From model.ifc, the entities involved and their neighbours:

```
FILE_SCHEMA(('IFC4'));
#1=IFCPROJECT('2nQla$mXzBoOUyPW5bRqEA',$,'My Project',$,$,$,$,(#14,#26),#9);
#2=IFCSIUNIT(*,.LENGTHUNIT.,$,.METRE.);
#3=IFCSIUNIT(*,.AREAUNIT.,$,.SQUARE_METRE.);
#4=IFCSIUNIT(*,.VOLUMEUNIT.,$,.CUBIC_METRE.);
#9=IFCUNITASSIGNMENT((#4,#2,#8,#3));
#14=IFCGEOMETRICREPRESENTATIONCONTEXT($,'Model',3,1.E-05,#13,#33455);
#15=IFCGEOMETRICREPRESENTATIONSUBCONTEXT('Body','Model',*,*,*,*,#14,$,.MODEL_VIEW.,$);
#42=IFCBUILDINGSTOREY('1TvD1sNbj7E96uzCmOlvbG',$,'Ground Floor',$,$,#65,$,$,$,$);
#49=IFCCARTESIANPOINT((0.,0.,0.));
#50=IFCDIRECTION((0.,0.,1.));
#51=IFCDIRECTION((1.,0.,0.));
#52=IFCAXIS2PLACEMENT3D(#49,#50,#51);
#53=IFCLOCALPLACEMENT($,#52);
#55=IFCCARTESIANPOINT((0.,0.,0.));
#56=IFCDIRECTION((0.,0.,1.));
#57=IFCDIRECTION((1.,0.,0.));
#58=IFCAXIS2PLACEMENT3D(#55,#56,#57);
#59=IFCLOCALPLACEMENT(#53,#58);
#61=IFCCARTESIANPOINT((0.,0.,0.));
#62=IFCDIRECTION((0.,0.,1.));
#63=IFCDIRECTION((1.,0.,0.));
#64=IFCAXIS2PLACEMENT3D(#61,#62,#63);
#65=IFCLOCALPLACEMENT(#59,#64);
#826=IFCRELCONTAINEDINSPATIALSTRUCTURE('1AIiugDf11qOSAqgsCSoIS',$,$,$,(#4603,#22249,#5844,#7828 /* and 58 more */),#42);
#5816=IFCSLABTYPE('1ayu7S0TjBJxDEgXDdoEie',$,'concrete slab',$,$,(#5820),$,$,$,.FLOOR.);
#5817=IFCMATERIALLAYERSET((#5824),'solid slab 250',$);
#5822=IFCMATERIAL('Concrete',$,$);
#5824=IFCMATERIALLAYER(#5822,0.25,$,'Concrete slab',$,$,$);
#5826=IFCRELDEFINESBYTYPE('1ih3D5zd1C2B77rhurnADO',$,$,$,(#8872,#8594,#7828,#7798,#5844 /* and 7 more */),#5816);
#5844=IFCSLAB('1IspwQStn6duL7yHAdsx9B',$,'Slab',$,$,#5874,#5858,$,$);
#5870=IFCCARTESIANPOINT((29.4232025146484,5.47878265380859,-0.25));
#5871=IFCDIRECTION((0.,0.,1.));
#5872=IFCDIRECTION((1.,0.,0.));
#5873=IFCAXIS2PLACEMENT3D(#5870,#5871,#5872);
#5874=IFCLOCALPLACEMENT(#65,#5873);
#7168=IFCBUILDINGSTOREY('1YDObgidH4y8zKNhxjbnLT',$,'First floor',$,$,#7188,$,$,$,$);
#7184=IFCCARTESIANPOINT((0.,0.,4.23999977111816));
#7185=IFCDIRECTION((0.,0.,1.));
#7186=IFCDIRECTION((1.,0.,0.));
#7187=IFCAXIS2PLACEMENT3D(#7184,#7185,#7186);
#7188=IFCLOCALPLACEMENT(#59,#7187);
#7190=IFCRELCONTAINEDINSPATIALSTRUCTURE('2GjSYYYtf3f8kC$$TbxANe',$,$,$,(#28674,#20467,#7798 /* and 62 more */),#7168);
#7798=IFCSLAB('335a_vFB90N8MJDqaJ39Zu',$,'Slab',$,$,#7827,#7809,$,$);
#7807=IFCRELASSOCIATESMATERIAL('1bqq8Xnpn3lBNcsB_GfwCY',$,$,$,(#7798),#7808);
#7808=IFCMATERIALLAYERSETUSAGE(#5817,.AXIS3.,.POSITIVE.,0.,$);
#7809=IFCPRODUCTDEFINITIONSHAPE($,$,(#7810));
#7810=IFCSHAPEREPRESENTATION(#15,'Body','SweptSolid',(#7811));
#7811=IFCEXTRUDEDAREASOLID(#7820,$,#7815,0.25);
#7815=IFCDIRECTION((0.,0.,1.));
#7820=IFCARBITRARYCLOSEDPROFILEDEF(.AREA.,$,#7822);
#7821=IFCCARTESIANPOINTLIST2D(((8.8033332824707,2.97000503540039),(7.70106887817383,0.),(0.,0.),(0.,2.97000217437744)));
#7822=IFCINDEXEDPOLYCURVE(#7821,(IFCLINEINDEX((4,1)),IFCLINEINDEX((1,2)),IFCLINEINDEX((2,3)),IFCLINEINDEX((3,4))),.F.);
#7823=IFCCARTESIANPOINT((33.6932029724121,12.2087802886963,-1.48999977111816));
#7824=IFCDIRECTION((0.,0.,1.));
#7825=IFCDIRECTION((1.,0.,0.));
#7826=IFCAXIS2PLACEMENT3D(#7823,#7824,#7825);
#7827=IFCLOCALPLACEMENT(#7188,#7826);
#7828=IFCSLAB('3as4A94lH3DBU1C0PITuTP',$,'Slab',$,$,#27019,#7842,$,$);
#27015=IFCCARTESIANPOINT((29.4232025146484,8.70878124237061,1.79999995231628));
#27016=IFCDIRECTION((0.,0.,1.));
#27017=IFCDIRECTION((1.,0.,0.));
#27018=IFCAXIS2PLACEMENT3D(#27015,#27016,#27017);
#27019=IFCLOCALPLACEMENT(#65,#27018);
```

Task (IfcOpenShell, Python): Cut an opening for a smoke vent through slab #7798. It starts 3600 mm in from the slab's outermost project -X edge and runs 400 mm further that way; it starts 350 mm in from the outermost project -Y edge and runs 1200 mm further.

```python
import numpy as np
import ifcopenshell
import ifcopenshell.api.feature
import ifcopenshell.api.geometry
import ifcopenshell.api.root
import ifcopenshell.geom
import ifcopenshell.util.placement
import ifcopenshell.util.representation
import ifcopenshell.util.shape
import ifcopenshell.util.unit

model = ifcopenshell.open("model.ifc")
unit_scale = ifcopenshell.util.unit.calculate_unit_scale(model)
settings = ifcopenshell.geom.settings()


def volume(element):
    """Net volume in cubic metres, openings subtracted."""
    shape = ifcopenshell.geom.create_shape(settings, element)
    return ifcopenshell.util.shape.get_volume(shape.geometry)


slab = model.by_guid("335a_vFB90N8MJDqaJ39Zu")
before = volume(slab)

# Extent in the slab's own axes, in metres. The edges named are its -X and -Y sides.
slab_shape = ifcopenshell.geom.create_shape(settings, slab)
vertices = ifcopenshell.util.shape.get_vertices(slab_shape.geometry)
x_min, y_min, bottom = vertices.min(axis=0)
top = vertices[:, 2].max()

opening = ifcopenshell.api.root.create_entity(model, ifc_class="IfcOpeningElement", name="Smoke vent opening", predefined_type="OPENING")
context = ifcopenshell.util.representation.get_context(model, "Model", "Body", "MODEL_VIEW")
width, depth = 0.4, 1.2
outline = [(0.0, 0.0), (width, 0.0), (width, depth), (0.0, depth), (0.0, 0.0)]
# Overshoot both faces by 50 mm so the cut is clean.
shape = ifcopenshell.api.geometry.add_slab_representation(
    model, context=context, depth=top - bottom + 0.1, polyline=outline
)
ifcopenshell.api.geometry.assign_representation(model, product=opening, representation=shape)

matrix = ifcopenshell.util.placement.get_local_placement(slab.ObjectPlacement)
matrix[:, 3] = matrix @ np.append(np.array([x_min + 3.6, y_min + 0.35, bottom - 0.05]) / unit_scale, 1.0)
ifcopenshell.api.geometry.edit_object_placement(model, product=opening, matrix=matrix, is_si=False)
ifcopenshell.api.feature.add_feature(model, feature=opening, element=slab)

after = volume(slab)

print(f"slab volume {before:.3f} -> {after:.3f} m3")

model.write("model_edited.ifc")
```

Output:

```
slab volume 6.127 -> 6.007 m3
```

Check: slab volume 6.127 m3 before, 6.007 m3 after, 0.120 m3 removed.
